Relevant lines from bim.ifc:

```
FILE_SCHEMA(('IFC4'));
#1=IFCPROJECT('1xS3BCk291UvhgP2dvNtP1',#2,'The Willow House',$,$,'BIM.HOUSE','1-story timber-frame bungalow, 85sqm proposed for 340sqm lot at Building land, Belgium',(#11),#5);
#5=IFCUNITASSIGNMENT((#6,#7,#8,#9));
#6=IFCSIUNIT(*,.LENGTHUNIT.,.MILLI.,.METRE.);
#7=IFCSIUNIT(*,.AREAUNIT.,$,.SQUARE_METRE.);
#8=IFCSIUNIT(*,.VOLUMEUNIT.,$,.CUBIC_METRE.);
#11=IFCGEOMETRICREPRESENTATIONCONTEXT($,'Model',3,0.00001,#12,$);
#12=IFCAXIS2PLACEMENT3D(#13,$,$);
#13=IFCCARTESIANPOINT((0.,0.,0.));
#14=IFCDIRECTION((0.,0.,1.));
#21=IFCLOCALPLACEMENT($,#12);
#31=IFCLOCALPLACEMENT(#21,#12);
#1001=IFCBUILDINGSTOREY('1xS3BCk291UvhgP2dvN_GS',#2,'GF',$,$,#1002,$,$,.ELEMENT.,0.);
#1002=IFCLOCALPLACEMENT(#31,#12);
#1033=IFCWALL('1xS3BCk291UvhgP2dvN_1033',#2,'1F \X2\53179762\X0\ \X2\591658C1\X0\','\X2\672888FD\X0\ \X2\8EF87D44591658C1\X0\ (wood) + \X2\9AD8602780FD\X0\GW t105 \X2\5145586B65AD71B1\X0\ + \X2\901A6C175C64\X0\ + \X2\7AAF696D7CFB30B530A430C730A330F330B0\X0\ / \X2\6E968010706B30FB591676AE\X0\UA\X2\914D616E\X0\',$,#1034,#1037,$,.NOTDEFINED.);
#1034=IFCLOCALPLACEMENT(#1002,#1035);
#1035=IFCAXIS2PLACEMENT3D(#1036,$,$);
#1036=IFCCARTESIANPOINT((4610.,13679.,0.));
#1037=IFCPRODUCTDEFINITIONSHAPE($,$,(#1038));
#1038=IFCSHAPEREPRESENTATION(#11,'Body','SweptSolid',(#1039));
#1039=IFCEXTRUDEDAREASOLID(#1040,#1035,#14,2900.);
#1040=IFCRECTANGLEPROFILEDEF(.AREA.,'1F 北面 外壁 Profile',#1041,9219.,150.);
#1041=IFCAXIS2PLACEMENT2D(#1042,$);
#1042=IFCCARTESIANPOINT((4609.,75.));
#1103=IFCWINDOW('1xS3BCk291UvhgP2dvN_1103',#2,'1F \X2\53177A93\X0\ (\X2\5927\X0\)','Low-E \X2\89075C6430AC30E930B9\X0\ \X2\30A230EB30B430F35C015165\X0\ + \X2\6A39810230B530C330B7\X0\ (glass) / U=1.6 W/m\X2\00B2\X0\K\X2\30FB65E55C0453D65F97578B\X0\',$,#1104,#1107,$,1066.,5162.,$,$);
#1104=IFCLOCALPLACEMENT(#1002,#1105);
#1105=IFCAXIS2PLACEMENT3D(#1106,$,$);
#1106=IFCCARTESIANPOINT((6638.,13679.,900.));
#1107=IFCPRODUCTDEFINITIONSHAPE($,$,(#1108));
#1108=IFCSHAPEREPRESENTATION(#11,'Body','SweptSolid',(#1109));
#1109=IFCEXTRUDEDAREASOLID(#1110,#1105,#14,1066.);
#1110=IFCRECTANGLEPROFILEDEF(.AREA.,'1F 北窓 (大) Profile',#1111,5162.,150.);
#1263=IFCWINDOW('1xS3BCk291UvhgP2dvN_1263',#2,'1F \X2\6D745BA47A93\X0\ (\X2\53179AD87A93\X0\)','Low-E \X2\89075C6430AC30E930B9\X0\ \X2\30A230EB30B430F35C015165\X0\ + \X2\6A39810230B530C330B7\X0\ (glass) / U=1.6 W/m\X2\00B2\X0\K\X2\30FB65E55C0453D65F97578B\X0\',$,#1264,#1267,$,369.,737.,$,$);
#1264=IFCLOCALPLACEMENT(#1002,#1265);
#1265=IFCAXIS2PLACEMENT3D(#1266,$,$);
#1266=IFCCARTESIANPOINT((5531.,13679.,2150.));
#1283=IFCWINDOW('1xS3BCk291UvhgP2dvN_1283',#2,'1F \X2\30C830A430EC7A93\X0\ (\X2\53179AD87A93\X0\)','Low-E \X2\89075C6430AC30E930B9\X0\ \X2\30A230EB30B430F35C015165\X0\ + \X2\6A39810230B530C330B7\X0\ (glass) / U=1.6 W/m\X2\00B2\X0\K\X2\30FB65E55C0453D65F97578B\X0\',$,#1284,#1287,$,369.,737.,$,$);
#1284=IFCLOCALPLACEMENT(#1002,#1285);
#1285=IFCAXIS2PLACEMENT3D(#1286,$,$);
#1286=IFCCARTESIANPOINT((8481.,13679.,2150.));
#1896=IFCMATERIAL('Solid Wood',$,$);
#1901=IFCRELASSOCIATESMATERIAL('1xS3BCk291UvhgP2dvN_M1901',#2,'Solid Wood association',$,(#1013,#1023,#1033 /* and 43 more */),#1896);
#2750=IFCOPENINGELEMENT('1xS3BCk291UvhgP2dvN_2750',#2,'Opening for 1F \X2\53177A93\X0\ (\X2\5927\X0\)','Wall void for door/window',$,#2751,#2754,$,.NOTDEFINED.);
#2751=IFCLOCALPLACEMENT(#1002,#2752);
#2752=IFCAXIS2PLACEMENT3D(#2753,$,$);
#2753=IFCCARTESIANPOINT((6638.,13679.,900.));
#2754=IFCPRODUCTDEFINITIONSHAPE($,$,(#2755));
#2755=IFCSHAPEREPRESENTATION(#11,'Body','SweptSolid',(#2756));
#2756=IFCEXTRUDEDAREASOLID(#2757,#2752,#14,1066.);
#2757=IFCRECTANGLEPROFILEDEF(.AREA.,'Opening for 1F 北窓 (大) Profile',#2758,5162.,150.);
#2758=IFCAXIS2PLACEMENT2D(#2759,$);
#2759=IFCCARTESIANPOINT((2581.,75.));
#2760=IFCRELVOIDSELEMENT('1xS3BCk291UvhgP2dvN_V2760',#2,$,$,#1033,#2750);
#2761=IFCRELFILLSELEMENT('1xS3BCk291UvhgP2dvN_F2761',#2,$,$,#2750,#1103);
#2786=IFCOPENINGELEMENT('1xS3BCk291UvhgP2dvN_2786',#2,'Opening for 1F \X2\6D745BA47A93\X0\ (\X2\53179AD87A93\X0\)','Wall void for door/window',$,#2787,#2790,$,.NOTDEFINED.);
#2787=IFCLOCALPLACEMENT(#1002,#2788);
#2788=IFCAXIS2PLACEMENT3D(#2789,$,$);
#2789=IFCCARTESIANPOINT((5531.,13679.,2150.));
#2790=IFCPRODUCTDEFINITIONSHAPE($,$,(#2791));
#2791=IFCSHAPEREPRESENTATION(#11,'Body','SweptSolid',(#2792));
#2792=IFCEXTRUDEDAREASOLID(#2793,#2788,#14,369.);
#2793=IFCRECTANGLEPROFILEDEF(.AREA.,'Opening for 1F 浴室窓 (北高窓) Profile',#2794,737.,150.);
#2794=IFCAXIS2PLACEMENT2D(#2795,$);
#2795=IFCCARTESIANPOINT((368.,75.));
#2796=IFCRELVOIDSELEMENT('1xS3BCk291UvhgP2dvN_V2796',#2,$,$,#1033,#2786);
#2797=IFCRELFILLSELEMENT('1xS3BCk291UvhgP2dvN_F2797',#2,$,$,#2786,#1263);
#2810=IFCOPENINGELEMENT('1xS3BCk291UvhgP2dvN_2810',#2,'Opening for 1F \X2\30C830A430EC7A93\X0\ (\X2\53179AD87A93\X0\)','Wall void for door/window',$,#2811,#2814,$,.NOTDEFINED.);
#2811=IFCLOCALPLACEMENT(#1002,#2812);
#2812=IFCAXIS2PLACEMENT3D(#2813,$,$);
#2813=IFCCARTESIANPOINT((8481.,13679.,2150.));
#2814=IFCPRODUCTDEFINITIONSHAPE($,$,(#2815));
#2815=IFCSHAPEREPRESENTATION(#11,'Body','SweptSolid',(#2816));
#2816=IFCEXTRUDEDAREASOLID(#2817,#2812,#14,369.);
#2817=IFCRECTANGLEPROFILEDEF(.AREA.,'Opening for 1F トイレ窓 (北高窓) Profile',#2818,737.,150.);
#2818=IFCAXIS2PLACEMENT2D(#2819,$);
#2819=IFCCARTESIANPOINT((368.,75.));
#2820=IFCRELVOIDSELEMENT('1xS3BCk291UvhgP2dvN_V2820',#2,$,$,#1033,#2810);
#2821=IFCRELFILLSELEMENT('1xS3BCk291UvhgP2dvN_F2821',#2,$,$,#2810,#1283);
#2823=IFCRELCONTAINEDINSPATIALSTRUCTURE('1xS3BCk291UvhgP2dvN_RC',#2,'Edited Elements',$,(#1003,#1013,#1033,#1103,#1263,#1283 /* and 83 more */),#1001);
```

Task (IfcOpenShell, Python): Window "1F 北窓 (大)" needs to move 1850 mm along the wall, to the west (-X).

```python
import ifcopenshell
import ifcopenshell.api.geometry
import ifcopenshell.util.placement
import ifcopenshell.util.unit

model = ifcopenshell.open("bim.ifc")
unit_scale = ifcopenshell.util.unit.calculate_unit_scale(model)

window = model.by_id(1103)
opening = window.FillsVoids[0].RelatingOpeningElement
wall = opening.VoidsElements[0].RelatingBuildingElement

wall_matrix = ifcopenshell.util.placement.get_local_placement(wall.ObjectPlacement)
shift = wall_matrix[:3, 0] * -1.85 / unit_scale
before = ifcopenshell.util.placement.get_local_placement(window.ObjectPlacement)[:3, 3].copy()

# The window is not placed relative to its opening, so move both.
for product in (opening, window):
    matrix = ifcopenshell.util.placement.get_local_placement(product.ObjectPlacement)
    matrix[:3, 3] += shift
    ifcopenshell.api.geometry.edit_object_placement(model, product=product, matrix=matrix, is_si=False)

after = ifcopenshell.util.placement.get_local_placement(window.ObjectPlacement)[:3, 3]
print("window moved by", (after - before).round(3) + 0.0)

model.write("bim_updated.ifc")
```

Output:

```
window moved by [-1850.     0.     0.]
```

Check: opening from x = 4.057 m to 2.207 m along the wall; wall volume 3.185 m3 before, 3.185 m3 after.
